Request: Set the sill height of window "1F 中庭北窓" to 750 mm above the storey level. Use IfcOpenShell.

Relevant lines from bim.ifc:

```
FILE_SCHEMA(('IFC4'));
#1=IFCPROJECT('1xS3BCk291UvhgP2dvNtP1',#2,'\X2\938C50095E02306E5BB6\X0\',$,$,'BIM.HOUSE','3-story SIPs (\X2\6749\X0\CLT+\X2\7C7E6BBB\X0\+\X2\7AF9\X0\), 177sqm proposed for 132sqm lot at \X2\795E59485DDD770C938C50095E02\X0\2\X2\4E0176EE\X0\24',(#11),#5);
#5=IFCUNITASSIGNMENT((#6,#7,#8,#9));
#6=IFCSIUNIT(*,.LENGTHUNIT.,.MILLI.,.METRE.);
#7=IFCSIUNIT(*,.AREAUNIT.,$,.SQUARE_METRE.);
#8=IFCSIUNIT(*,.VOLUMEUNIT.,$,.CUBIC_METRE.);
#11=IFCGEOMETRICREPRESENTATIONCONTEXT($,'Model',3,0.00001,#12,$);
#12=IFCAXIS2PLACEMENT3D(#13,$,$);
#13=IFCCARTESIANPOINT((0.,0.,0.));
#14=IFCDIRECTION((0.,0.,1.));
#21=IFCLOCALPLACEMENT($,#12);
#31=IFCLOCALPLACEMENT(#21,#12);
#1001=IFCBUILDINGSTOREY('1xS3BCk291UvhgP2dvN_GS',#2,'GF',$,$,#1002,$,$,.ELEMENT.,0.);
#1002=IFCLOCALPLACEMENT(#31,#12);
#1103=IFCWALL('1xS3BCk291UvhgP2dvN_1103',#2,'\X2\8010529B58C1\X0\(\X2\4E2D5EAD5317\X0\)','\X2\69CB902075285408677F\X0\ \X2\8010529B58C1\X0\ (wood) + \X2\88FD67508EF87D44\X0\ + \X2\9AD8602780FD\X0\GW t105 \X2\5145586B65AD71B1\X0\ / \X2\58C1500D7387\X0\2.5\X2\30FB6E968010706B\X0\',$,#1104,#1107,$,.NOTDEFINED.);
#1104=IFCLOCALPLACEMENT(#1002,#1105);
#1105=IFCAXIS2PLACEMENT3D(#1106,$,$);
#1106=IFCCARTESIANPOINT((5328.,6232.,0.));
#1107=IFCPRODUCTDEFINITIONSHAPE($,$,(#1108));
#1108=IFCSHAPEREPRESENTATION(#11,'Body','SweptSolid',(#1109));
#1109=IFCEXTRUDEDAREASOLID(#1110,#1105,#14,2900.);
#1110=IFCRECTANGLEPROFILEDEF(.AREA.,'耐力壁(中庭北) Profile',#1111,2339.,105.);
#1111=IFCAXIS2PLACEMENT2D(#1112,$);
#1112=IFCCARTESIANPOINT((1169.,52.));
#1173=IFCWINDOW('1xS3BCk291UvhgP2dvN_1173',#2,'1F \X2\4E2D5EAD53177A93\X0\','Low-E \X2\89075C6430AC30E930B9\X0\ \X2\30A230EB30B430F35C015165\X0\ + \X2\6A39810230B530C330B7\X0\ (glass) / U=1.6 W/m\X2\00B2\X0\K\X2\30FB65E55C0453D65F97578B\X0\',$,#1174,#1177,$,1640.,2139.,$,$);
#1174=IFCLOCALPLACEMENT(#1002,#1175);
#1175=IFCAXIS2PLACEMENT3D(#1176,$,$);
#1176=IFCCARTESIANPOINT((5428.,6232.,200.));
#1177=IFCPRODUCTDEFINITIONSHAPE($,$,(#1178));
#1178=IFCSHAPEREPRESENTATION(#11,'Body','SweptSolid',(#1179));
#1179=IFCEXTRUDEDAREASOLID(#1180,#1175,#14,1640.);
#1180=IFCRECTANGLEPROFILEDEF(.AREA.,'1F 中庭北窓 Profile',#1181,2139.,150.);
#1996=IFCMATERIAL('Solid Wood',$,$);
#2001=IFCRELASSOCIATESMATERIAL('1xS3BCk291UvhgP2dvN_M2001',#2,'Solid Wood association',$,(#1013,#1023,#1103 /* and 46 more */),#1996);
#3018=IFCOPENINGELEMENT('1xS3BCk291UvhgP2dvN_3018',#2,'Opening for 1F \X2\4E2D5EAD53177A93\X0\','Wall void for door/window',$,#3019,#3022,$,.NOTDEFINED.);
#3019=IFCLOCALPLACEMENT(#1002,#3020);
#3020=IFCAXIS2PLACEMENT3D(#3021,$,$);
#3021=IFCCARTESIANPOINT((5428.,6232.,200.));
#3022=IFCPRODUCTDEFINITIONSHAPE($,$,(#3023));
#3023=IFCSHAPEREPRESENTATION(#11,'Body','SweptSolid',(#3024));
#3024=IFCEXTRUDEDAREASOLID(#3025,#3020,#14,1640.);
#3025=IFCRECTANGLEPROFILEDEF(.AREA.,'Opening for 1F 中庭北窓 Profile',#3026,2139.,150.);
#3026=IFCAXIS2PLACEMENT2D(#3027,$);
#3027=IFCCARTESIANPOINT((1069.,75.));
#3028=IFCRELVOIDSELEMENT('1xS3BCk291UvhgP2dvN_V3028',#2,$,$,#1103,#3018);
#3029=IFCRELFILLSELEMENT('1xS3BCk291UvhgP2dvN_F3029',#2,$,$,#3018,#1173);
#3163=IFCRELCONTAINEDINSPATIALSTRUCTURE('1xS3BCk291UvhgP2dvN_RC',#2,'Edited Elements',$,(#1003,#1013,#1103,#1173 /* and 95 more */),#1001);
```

```python
import numpy as np
import ifcopenshell
import ifcopenshell.api.geometry
import ifcopenshell.geom
import ifcopenshell.util.element
import ifcopenshell.util.placement
import ifcopenshell.util.shape
import ifcopenshell.util.unit

model = ifcopenshell.open("bim.ifc")
unit_scale = ifcopenshell.util.unit.calculate_unit_scale(model)

window = model.by_id(1173)
opening = window.FillsVoids[0].RelatingOpeningElement
storey = ifcopenshell.util.element.get_container(window, ifc_class="IfcBuildingStorey")
level = ifcopenshell.util.placement.get_local_placement(storey.ObjectPlacement)[2, 3]

# The opening's origin need not be at the sill, so measure its lowest point.
shape = ifcopenshell.geom.create_shape(ifcopenshell.geom.settings(), opening)
bottom = ifcopenshell.util.shape.get_shape_bottom_elevation(shape, shape.geometry) / unit_scale
dz = level + 0.75 / unit_scale - bottom

shift = np.array([0.0, 0.0, dz])
# The window is not placed relative to its opening, so move both.
for product in (opening, window):
    matrix = ifcopenshell.util.placement.get_local_placement(product.ObjectPlacement)
    matrix[:3, 3] += shift
    ifcopenshell.api.geometry.edit_object_placement(model, product=product, matrix=matrix, is_si=False)

print(f"moved by {dz * unit_scale:+.3f} m")

model.write("bim_rev.ifc")
```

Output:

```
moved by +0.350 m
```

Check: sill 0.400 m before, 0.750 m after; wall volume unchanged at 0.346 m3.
